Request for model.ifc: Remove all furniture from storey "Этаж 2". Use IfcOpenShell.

First a look at what the model holds.

```python
import ifcopenshell
import ifcopenshell.util.element

model = ifcopenshell.open("model.ifc")
print(model.schema)
storey = next(s for s in model.by_type("IfcBuildingStorey") if s.Name == "Этаж 2")
furniture = [e for e in ifcopenshell.util.element.get_decomposition(storey) if e.is_a("IfcFurnishingElement")]
seen = {}
for e in furniture:
    element_type = ifcopenshell.util.element.get_type(e)
    name = element_type.Name if element_type not in (None, e) else None
    seen[name] = seen.get(name, 0) + 1
for name, count in sorted(seen.items(), key=str):
    print(count, "x", name)
```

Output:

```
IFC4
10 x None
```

```python
import ifcopenshell
import ifcopenshell.api.root
import ifcopenshell.util.element

model = ifcopenshell.open("model.ifc")

storey = next(s for s in model.by_type("IfcBuildingStorey") if s.Name == "Этаж 2")
furniture = [e for e in ifcopenshell.util.element.get_decomposition(storey) if e.is_a("IfcFurnishingElement")]

for e in furniture:
    ifcopenshell.api.root.remove_product(model, product=e)
print(len(furniture), "removed")

model.write("model_v2.ifc")
```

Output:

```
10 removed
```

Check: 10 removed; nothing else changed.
